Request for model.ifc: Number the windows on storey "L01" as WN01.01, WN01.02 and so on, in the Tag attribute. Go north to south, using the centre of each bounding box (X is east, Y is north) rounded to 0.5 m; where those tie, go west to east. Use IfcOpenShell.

First a look at what the model holds.

```python
import ifcopenshell
import ifcopenshell.util.element
import ifcopenshell.util.placement

model = ifcopenshell.open("model.ifc")
print(model.schema)
storey = next(s for s in model.by_type("IfcBuildingStorey") if s.Name == "L01")
windows = [e for e in ifcopenshell.util.element.get_decomposition(storey) if e.is_a("IfcWindow")]
for e in sorted(windows, key=lambda e: e.id()):
    origin = ifcopenshell.util.placement.get_local_placement(e.ObjectPlacement)[:3, 3]
    print(e.id(), e.Tag, e.Name, origin.round(2) + 0.0, sep=" | ")
```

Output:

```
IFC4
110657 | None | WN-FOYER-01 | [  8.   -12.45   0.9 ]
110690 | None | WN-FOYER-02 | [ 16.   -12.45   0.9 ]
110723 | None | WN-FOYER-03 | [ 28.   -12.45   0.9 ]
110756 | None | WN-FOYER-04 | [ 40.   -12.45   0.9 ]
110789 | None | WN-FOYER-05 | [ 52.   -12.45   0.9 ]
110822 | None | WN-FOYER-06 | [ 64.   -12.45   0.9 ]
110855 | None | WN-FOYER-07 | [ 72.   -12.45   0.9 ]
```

```python
import ifcopenshell
import ifcopenshell.geom
import ifcopenshell.util.element
import ifcopenshell.util.shape

model = ifcopenshell.open("model.ifc")
settings = ifcopenshell.geom.settings()
settings.set("use-world-coords", True)


def centre(element):
    shape = ifcopenshell.geom.create_shape(settings, element)
    return ifcopenshell.util.shape.get_bbox_centroid(shape.geometry)


storey = next(s for s in model.by_type("IfcBuildingStorey") if s.Name == "L01")
windows = [e for e in ifcopenshell.util.element.get_decomposition(storey) if e.is_a("IfcWindow")]

# Insertion points can sit at a corner or the storey origin, so sort by the geometry (in metres).
centres = {e: centre(e) for e in windows}
windows.sort(key=lambda e: (-round(centres[e][1] / 0.5), centres[e][0]))

for i, e in enumerate(windows, start=1):
    number = f"WN01.{i:02d}"
    e.Tag = number
    print(e.id(), number)

model.write("model-out.ifc")
```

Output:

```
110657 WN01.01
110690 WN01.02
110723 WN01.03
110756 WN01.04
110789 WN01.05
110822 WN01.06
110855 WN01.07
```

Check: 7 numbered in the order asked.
